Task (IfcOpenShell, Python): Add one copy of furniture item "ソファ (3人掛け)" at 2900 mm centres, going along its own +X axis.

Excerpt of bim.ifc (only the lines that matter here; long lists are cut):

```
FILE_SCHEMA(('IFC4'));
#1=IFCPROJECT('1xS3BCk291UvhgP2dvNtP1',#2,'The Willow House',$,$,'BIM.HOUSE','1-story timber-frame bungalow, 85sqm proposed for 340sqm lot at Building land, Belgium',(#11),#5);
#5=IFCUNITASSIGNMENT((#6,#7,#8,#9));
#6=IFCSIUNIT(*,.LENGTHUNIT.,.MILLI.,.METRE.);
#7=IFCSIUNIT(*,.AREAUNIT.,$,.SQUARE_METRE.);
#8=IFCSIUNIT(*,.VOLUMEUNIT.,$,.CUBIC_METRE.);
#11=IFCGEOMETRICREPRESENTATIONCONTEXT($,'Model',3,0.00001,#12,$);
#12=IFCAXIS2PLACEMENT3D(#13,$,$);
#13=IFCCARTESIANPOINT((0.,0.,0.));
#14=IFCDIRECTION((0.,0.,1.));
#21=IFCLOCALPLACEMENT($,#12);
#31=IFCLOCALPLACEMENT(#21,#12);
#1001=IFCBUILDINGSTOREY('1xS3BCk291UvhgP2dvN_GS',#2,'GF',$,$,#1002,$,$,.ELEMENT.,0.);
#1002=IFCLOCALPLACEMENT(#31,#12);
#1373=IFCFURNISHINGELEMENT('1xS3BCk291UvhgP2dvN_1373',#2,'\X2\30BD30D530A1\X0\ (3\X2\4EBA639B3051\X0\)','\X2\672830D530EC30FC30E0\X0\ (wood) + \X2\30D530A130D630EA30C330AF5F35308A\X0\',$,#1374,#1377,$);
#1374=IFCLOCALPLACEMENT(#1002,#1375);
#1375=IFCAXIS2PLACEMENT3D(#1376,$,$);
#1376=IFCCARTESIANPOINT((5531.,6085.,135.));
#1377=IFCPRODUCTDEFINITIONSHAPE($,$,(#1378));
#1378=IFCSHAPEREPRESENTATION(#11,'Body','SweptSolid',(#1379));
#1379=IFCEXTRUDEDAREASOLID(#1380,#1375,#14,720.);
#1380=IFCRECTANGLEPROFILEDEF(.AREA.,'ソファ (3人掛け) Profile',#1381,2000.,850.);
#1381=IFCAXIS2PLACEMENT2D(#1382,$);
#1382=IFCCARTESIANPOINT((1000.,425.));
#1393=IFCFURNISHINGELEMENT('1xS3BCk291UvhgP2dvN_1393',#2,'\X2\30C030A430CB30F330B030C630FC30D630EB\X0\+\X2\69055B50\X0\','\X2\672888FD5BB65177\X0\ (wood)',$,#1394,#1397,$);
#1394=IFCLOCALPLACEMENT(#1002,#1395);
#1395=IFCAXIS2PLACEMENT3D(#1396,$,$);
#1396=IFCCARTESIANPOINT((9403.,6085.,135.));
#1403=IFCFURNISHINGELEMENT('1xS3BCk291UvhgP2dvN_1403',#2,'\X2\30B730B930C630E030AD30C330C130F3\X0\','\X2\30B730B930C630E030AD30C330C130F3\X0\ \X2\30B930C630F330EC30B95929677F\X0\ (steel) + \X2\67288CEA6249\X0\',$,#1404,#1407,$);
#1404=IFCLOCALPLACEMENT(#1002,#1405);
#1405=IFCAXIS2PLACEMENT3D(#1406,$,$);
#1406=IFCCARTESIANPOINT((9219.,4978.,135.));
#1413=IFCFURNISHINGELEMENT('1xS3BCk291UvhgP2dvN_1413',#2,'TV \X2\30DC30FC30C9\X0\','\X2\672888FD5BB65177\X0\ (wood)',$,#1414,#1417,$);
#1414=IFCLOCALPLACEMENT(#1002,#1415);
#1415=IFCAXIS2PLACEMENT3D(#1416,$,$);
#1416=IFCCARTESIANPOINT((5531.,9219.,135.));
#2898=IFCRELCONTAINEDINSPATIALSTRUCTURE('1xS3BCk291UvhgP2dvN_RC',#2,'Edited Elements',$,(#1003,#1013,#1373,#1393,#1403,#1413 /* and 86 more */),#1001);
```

```python
import ifcopenshell
import ifcopenshell.api.geometry
import ifcopenshell.api.root
import ifcopenshell.util.element
import ifcopenshell.util.placement
import ifcopenshell.util.unit

model = ifcopenshell.open("bim.ifc")
unit_scale = ifcopenshell.util.unit.calculate_unit_scale(model)


def reuse_history(source, copy):
    """copy_class also copies each property set's owner history, people and application; keep the originals."""
    for rel in copy.IsDefinedBy:
        if rel.is_a("IfcRelDefinesByProperties") and (history := rel.RelatingPropertyDefinition.OwnerHistory):
            rel.RelatingPropertyDefinition.OwnerHistory = source.OwnerHistory
            ifcopenshell.util.element.remove_deep2(model, history)


source = model.by_guid("1xS3BCk291UvhgP2dvN_1373")
base = ifcopenshell.util.placement.get_local_placement(source.ObjectPlacement)
step = base[:3, 0] * 2.9 / unit_scale

for i in range(1, 2):
    copy = ifcopenshell.api.root.copy_class(model, product=source)
    copy.Representation = ifcopenshell.util.element.copy_deep(
        model, source.Representation, exclude=["IfcGeometricRepresentationContext", "IfcRepresentationMap"]
    )
    reuse_history(source, copy)
    matrix = base.copy()
    matrix[:3, 3] += i * step
    print("added at", matrix[:3, 3].round(3) + 0.0)
    ifcopenshell.api.geometry.edit_object_placement(model, product=copy, matrix=matrix, is_si=False)

model.write("bim_edited.ifc")
```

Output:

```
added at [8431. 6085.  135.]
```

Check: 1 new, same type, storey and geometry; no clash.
